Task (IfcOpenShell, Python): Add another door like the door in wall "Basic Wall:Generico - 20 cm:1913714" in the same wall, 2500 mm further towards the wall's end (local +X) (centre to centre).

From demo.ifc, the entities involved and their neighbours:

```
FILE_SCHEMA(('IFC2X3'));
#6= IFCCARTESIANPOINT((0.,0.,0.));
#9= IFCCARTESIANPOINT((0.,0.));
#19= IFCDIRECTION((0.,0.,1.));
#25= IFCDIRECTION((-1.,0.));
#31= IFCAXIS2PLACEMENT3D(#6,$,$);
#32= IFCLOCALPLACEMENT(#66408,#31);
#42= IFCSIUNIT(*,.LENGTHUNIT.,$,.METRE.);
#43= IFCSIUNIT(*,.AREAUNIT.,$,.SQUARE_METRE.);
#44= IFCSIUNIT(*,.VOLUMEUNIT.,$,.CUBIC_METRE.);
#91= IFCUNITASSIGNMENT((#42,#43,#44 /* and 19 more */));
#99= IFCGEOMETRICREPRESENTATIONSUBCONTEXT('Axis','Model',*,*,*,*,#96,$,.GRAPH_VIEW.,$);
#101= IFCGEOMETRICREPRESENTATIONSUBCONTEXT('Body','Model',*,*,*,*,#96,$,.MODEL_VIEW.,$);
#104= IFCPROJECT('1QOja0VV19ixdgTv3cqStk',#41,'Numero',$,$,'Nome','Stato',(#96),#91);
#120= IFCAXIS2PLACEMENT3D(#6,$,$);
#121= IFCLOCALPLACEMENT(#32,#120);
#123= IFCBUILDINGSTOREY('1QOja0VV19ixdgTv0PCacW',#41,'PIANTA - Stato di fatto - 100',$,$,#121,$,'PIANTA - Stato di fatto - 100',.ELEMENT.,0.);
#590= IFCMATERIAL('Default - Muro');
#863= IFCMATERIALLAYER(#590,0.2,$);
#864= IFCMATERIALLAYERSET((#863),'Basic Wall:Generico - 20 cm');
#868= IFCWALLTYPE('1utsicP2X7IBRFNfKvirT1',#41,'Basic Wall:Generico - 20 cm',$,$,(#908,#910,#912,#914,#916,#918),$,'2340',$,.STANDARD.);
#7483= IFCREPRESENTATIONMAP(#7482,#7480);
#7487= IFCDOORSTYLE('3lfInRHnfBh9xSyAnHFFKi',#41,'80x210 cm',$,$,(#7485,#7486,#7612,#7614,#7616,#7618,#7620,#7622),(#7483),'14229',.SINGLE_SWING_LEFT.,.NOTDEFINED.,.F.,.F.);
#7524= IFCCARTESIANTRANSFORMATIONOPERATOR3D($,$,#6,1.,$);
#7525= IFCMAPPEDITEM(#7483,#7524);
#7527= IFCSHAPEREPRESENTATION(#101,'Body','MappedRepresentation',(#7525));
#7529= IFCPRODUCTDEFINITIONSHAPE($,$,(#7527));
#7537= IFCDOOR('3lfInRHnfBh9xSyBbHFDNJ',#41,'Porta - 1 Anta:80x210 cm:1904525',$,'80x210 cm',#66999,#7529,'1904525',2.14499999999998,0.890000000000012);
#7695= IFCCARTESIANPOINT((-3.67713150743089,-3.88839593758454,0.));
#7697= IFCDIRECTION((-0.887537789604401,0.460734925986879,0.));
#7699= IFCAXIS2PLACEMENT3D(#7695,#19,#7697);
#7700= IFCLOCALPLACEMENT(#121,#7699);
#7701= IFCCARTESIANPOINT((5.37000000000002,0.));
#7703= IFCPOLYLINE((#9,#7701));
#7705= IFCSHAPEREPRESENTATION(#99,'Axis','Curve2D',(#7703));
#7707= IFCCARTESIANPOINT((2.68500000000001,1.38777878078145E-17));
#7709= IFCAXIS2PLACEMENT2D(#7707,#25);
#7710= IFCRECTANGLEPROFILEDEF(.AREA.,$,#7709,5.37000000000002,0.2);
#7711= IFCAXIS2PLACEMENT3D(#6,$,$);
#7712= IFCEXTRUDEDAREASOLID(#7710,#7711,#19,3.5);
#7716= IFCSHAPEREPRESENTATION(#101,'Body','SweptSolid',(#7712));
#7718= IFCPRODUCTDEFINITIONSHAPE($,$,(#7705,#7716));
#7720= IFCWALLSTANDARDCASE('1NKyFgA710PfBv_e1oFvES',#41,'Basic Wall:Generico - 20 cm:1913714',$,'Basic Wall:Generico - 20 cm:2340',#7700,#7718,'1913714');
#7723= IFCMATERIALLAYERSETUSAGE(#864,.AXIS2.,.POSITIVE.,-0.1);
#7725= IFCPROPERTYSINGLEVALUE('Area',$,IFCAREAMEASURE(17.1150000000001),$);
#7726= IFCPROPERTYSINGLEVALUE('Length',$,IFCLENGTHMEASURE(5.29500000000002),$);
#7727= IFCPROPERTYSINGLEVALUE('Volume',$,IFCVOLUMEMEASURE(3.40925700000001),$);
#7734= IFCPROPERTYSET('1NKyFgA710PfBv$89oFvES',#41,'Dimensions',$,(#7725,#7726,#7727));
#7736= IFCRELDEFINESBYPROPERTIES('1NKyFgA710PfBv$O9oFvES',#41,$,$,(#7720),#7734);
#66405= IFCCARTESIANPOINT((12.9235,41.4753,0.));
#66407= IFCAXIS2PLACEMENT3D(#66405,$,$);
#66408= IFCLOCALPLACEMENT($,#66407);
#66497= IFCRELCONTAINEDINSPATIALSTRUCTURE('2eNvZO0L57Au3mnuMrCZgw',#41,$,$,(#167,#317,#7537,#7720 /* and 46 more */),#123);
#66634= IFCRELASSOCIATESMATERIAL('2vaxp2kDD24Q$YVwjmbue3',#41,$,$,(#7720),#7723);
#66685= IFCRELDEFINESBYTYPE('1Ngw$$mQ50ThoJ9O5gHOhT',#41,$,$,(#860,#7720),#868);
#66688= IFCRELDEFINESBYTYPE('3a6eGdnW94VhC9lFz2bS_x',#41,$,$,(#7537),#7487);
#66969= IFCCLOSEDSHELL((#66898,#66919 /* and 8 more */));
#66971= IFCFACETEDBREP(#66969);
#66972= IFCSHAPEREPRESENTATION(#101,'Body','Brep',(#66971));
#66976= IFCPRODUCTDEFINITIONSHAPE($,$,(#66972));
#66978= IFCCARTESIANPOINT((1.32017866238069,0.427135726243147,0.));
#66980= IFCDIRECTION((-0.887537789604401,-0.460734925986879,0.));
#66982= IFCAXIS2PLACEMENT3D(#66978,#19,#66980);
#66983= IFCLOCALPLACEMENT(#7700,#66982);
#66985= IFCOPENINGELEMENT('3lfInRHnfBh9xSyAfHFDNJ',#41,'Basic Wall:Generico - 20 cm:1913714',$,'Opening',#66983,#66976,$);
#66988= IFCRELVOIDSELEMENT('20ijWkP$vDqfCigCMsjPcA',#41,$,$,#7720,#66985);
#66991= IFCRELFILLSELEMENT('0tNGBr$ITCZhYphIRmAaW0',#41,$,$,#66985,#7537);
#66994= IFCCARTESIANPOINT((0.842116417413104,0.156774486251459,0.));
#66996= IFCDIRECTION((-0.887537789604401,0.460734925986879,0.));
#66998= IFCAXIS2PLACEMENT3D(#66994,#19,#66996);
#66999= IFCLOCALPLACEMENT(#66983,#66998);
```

```python
import ifcopenshell
import ifcopenshell.api.feature
import ifcopenshell.api.geometry
import ifcopenshell.api.pset
import ifcopenshell.api.root
import ifcopenshell.geom
import ifcopenshell.util.element
import ifcopenshell.util.placement
import ifcopenshell.util.shape
import ifcopenshell.util.unit

model = ifcopenshell.open("demo.ifc")
area_scale = ifcopenshell.util.unit.calculate_unit_scale(model, "AREAUNIT")
volume_scale = ifcopenshell.util.unit.calculate_unit_scale(model, "VOLUMEUNIT")
settings = ifcopenshell.geom.settings()


def volume(element):
    """Net volume in cubic metres, openings subtracted."""
    shape = ifcopenshell.geom.create_shape(settings, element)
    return ifcopenshell.util.shape.get_volume(shape.geometry)


def reuse_history(source, copy):
    """copy_class also copies each property set's owner history, people and application; keep the originals."""
    for rel in copy.IsDefinedBy:
        if rel.is_a("IfcRelDefinesByProperties") and (history := rel.RelatingPropertyDefinition.OwnerHistory):
            rel.RelatingPropertyDefinition.OwnerHistory = source.OwnerHistory
            ifcopenshell.util.element.remove_deep2(model, history)


door = model.by_guid("3lfInRHnfBh9xSyBbHFDNJ")
opening = door.FillsVoids[0].RelatingOpeningElement
wall = opening.VoidsElements[0].RelatingBuildingElement
before = volume(wall)
shift = ifcopenshell.util.placement.get_local_placement(wall.ObjectPlacement)[:3, 0] * 2.5

# copy_class copies the void relationship, type, container and properties, but no geometry.
new_opening = ifcopenshell.api.root.copy_class(model, product=opening)
new_opening.Representation = ifcopenshell.util.element.copy_deep(
    model, opening.Representation, exclude=["IfcGeometricRepresentationContext", "IfcRepresentationMap"]
)
new_opening.Name = "Basic Wall:Generico - 20 cm"
new_door = ifcopenshell.api.root.copy_class(model, product=door)
new_door.Representation = ifcopenshell.util.element.copy_deep(
    model, door.Representation, exclude=["IfcGeometricRepresentationContext", "IfcRepresentationMap"]
)
new_door.Name = "Porta - 1 Anta:80x210 cm"
new_door.Tag = None
reuse_history(door, new_door)
fills = ifcopenshell.api.feature.add_filling(model, opening=new_opening, element=new_door)
fills.OwnerHistory = new_door.OwnerHistory  # required in IFC2X3

for old, new in ((opening, new_opening), (door, new_door)):
    matrix = ifcopenshell.util.placement.get_local_placement(old.ObjectPlacement)
    matrix[:3, 3] += shift
    ifcopenshell.api.geometry.edit_object_placement(model, product=new, matrix=matrix, is_si=False)

after = volume(wall)
thickness = 0.2  # wall thickness in metres

# Update the wall's stored quantities.
pset = model.by_id(ifcopenshell.util.element.get_pset(wall, "Dimensions", should_inherit=False)["id"])
ifcopenshell.api.pset.edit_pset(model, pset=pset, properties={
    "Area": model.create_entity("IfcAreaMeasure", after / thickness / area_scale),
    "Volume": model.create_entity("IfcVolumeMeasure", after / volume_scale),
})

print(f"wall volume {before:.3f} -> {after:.3f} m3")

model.write("demo_edited.ifc")
```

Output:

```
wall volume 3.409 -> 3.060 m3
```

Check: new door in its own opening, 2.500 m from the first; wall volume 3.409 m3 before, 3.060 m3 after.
